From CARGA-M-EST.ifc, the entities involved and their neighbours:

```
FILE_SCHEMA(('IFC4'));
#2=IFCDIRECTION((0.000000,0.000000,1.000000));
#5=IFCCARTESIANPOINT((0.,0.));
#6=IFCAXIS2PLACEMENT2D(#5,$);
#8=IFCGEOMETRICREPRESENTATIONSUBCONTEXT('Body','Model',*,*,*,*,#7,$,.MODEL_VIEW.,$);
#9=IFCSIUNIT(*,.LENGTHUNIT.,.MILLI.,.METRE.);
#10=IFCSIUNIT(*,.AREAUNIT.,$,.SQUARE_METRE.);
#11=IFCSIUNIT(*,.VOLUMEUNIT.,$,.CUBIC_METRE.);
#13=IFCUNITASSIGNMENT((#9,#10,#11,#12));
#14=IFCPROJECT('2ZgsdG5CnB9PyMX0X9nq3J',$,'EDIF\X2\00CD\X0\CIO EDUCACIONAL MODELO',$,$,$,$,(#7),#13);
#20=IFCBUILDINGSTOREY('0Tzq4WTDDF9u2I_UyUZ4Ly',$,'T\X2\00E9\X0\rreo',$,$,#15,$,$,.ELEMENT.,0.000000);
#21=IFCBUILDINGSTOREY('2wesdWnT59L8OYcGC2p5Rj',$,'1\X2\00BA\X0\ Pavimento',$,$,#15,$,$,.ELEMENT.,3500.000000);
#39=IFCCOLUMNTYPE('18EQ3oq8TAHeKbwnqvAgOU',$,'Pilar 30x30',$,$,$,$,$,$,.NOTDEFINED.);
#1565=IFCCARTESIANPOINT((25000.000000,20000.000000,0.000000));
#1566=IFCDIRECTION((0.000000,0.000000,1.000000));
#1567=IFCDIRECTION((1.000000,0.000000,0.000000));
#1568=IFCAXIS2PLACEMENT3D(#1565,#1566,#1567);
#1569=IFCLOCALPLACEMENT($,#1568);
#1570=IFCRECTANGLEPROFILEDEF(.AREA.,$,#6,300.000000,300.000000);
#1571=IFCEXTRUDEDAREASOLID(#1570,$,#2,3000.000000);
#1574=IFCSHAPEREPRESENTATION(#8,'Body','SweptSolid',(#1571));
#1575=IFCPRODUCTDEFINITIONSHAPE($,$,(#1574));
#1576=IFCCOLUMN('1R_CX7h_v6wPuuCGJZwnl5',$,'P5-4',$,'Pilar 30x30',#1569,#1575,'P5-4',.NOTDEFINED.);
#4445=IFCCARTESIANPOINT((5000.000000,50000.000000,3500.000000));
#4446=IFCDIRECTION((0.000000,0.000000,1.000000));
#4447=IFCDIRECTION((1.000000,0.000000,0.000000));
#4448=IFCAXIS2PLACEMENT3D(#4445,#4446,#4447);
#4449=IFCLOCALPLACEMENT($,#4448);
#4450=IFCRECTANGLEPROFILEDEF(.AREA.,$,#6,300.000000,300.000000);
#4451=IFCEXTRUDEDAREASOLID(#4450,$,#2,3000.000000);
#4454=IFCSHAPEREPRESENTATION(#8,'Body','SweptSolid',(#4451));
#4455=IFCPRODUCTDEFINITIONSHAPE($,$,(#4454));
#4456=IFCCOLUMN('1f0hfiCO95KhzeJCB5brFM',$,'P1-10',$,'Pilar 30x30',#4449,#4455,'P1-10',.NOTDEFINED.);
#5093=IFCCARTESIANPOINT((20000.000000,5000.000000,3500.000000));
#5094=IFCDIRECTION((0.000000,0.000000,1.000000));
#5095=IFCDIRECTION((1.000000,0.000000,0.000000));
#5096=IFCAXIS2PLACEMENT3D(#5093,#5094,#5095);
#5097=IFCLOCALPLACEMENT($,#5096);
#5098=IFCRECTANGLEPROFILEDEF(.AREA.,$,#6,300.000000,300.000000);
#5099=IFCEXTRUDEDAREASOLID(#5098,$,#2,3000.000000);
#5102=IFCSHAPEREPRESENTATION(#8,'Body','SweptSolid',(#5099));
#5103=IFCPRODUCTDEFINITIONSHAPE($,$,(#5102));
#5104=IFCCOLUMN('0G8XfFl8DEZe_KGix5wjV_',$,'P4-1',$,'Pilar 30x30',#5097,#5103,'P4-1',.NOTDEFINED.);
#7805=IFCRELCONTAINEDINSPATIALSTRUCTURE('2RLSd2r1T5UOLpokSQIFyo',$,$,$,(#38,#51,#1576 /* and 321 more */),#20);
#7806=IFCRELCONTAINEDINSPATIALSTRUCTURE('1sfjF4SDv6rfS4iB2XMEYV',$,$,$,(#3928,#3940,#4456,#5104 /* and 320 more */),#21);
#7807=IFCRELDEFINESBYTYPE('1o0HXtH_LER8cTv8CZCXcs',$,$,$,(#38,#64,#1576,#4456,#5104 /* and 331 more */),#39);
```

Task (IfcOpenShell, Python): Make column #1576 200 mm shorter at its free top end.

```python
import ifcopenshell
import ifcopenshell.util.representation

model = ifcopenshell.open("CARGA-M-EST.ifc")

member = model.by_guid("1R_CX7h_v6wPuuCGJZwnl5")
change = -200.0

# The extrusion runs towards the end named, so only its depth changes.
body = ifcopenshell.util.representation.get_representation(member, "Model", "Body")
solid = body.Items[0]
old_length = solid.Depth
solid.Depth += change

print(f"length {old_length:g} -> {solid.Depth:g}")

model.write("CARGA-M-EST_rev.ifc")
```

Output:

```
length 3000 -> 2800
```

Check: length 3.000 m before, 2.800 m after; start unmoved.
